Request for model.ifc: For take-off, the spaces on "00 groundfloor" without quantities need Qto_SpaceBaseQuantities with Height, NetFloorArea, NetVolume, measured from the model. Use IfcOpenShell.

First a look at what the model holds.

```python
import ifcopenshell
import ifcopenshell.util.element
import ifcopenshell.util.unit

model = ifcopenshell.open("model.ifc")
print(model.schema)
for unit_type in ("LENGTHUNIT", "AREAUNIT", "VOLUMEUNIT"):
    print(unit_type, ifcopenshell.util.unit.calculate_unit_scale(model, unit_type))
storey = next(s for s in model.by_type("IfcBuildingStorey") if s.Name == "00 groundfloor")
spaces = [e for e in ifcopenshell.util.element.get_decomposition(storey) if e.is_a("IfcSpace")]
for e in sorted(spaces, key=lambda e: e.id()):
    print(e.id(), e.is_a(), e.Name, list(ifcopenshell.util.element.get_psets(e, qtos_only=True)), sep=" | ")
```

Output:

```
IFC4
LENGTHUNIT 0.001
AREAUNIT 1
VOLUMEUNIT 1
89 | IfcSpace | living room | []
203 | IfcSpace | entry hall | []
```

```python
import ifcopenshell
import ifcopenshell.api.pset
import ifcopenshell.geom
import ifcopenshell.util.element
import ifcopenshell.util.shape
import ifcopenshell.util.unit

model = ifcopenshell.open("model.ifc")
unit_scale = ifcopenshell.util.unit.calculate_unit_scale(model)
area_scale = ifcopenshell.util.unit.calculate_unit_scale(model, "AREAUNIT")
volume_scale = ifcopenshell.util.unit.calculate_unit_scale(model, "VOLUMEUNIT")
settings = ifcopenshell.geom.settings()

storey = next(s for s in model.by_type("IfcBuildingStorey") if s.Name == "00 groundfloor")
spaces = [e for e in ifcopenshell.util.element.get_decomposition(storey) if e.is_a("IfcSpace")]

for e in sorted(spaces, key=lambda e: e.id()):
    if ifcopenshell.util.element.get_psets(e, qtos_only=True, should_inherit=False):
        continue
    # Geometry comes back in metres, in the element's own axes.
    shape = ifcopenshell.geom.create_shape(settings, e)
    values = {
        "Height": ifcopenshell.util.shape.get_z(shape.geometry) / unit_scale,
        "NetFloorArea": ifcopenshell.util.shape.get_footprint_area(shape.geometry) / area_scale,
        "NetVolume": ifcopenshell.util.shape.get_volume(shape.geometry) / volume_scale,
    }
    qto = ifcopenshell.api.pset.add_qto(model, product=e, name="Qto_SpaceBaseQuantities")
    ifcopenshell.api.pset.edit_qto(model, qto=qto, properties=values)
    print(e.id(), {k: round(v, 3) for k, v in values.items()})

model.write("model_rev.ifc")
```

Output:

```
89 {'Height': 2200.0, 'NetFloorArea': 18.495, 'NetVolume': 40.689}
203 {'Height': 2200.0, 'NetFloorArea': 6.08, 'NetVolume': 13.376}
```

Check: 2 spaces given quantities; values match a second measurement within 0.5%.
